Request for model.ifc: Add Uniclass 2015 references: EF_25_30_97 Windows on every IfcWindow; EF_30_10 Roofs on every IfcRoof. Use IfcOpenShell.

First a look at what the model holds.

```python
import ifcopenshell

model = ifcopenshell.open("model.ifc")
print(model.schema)
print("classifications:", [c.Name for c in model.by_type("IfcClassification")])
for ifc_class in ("IfcDoor", "IfcRoof", "IfcStair", "IfcWall", "IfcWindow"):
    print(ifc_class, len(model.by_type(ifc_class)))
```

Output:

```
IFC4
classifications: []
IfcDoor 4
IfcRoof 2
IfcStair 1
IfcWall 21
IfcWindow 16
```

```python
import ifcopenshell
import ifcopenshell.api.classification

model = ifcopenshell.open("model.ifc")

system = ifcopenshell.api.classification.add_classification(model, classification="Uniclass 2015")

codes = {
    "IfcWindow": ("EF_25_30_97", "Windows"),
    "IfcRoof": ("EF_30_10", "Roofs"),
}
for ifc_class, (code, name) in codes.items():
    products = model.by_type(ifc_class)
    ifcopenshell.api.classification.add_reference(
        model, products=products, classification=system, identification=code, name=name
    )
    print(code, len(products))

model.write("model_updated.ifc")
```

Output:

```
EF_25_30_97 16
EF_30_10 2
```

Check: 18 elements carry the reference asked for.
